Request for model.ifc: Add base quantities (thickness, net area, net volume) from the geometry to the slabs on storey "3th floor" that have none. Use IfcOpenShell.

First a look at what the model holds.

```python
import ifcopenshell
import ifcopenshell.util.element
import ifcopenshell.util.unit

model = ifcopenshell.open("model.ifc")
print(model.schema)
for unit_type in ("LENGTHUNIT", "AREAUNIT", "VOLUMEUNIT"):
    print(unit_type, ifcopenshell.util.unit.calculate_unit_scale(model, unit_type))
storey = next(s for s in model.by_type("IfcBuildingStorey") if s.Name == "3th floor")
slabs = [e for e in ifcopenshell.util.element.get_decomposition(storey) if e.is_a("IfcSlab")]
for e in sorted(slabs, key=lambda e: e.id()):
    print(e.id(), e.is_a(), e.Name, list(ifcopenshell.util.element.get_psets(e, qtos_only=True)), sep=" | ")
```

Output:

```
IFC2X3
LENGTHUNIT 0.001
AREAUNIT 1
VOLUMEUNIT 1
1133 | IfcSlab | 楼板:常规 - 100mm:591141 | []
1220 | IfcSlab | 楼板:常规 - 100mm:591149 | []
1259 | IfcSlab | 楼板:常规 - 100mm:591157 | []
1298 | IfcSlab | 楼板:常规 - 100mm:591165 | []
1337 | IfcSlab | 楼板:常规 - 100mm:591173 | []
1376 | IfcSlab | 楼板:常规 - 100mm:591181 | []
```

```python
import ifcopenshell
import ifcopenshell.api.pset
import ifcopenshell.geom
import ifcopenshell.util.element
import ifcopenshell.util.shape
import ifcopenshell.util.unit

model = ifcopenshell.open("model.ifc")
unit_scale = ifcopenshell.util.unit.calculate_unit_scale(model)
area_scale = ifcopenshell.util.unit.calculate_unit_scale(model, "AREAUNIT")
volume_scale = ifcopenshell.util.unit.calculate_unit_scale(model, "VOLUMEUNIT")
settings = ifcopenshell.geom.settings()

storey = next(s for s in model.by_type("IfcBuildingStorey") if s.Name == "3th floor")
slabs = [e for e in ifcopenshell.util.element.get_decomposition(storey) if e.is_a("IfcSlab")]

for e in sorted(slabs, key=lambda e: e.id()):
    if ifcopenshell.util.element.get_psets(e, qtos_only=True, should_inherit=False):
        continue
    # Geometry comes back in metres, in the element's own axes.
    shape = ifcopenshell.geom.create_shape(settings, e)
    values = {
        "Width": ifcopenshell.util.shape.get_z(shape.geometry) / unit_scale,
        "NetArea": ifcopenshell.util.shape.get_footprint_area(shape.geometry) / area_scale,
        "NetVolume": ifcopenshell.util.shape.get_volume(shape.geometry) / volume_scale,
    }
    qto = ifcopenshell.api.pset.add_qto(model, product=e, name="BaseQuantities")
    ifcopenshell.api.pset.edit_qto(model, qto=qto, properties=values)
    print(e.id(), {k: round(v, 3) for k, v in values.items()})

model.write("model_edited.ifc")
```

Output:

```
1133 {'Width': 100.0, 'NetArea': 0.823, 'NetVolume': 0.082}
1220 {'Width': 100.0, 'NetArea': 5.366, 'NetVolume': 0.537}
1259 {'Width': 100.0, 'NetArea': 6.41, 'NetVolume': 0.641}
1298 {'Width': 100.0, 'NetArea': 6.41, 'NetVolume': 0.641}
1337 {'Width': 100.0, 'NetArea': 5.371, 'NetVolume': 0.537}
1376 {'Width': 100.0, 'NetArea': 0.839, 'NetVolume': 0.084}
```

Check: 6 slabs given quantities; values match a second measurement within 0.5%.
